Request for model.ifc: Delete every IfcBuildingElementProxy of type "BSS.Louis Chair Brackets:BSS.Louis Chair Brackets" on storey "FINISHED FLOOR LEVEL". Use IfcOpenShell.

First a look at what the model holds.

```python
import ifcopenshell
import ifcopenshell.util.element

model = ifcopenshell.open("model.ifc")
print(model.schema)
storey = next(s for s in model.by_type("IfcBuildingStorey") if s.Name == "FINISHED FLOOR LEVEL")
proxies = [e for e in ifcopenshell.util.element.get_decomposition(storey) if e.is_a("IfcBuildingElementProxy")]
seen = {}
for e in proxies:
    element_type = ifcopenshell.util.element.get_type(e)
    name = element_type.Name if element_type not in (None, e) else None
    seen[name] = seen.get(name, 0) + 1
for name, count in sorted(seen.items(), key=str):
    print(count, "x", name)
```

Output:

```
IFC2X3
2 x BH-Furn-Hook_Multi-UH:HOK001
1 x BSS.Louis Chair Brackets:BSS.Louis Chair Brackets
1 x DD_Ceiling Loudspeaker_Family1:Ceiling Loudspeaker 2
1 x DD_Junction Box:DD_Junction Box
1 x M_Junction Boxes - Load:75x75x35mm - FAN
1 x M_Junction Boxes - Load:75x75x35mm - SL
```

```python
import ifcopenshell
import ifcopenshell.api.root
import ifcopenshell.util.element

model = ifcopenshell.open("model.ifc")

storey = next(s for s in model.by_type("IfcBuildingStorey") if s.Name == "FINISHED FLOOR LEVEL")
proxies = [e for e in ifcopenshell.util.element.get_decomposition(storey) if e.is_a("IfcBuildingElementProxy")]
targets = [e for e in proxies if (t := ifcopenshell.util.element.get_type(e)) not in (None, e) and t.Name == "BSS.Louis Chair Brackets:BSS.Louis Chair Brackets"]

for e in targets:
    ifcopenshell.api.root.remove_product(model, product=e)
print(len(targets), "removed")

model.write("model_rev.ifc")
```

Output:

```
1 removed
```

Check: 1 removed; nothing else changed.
